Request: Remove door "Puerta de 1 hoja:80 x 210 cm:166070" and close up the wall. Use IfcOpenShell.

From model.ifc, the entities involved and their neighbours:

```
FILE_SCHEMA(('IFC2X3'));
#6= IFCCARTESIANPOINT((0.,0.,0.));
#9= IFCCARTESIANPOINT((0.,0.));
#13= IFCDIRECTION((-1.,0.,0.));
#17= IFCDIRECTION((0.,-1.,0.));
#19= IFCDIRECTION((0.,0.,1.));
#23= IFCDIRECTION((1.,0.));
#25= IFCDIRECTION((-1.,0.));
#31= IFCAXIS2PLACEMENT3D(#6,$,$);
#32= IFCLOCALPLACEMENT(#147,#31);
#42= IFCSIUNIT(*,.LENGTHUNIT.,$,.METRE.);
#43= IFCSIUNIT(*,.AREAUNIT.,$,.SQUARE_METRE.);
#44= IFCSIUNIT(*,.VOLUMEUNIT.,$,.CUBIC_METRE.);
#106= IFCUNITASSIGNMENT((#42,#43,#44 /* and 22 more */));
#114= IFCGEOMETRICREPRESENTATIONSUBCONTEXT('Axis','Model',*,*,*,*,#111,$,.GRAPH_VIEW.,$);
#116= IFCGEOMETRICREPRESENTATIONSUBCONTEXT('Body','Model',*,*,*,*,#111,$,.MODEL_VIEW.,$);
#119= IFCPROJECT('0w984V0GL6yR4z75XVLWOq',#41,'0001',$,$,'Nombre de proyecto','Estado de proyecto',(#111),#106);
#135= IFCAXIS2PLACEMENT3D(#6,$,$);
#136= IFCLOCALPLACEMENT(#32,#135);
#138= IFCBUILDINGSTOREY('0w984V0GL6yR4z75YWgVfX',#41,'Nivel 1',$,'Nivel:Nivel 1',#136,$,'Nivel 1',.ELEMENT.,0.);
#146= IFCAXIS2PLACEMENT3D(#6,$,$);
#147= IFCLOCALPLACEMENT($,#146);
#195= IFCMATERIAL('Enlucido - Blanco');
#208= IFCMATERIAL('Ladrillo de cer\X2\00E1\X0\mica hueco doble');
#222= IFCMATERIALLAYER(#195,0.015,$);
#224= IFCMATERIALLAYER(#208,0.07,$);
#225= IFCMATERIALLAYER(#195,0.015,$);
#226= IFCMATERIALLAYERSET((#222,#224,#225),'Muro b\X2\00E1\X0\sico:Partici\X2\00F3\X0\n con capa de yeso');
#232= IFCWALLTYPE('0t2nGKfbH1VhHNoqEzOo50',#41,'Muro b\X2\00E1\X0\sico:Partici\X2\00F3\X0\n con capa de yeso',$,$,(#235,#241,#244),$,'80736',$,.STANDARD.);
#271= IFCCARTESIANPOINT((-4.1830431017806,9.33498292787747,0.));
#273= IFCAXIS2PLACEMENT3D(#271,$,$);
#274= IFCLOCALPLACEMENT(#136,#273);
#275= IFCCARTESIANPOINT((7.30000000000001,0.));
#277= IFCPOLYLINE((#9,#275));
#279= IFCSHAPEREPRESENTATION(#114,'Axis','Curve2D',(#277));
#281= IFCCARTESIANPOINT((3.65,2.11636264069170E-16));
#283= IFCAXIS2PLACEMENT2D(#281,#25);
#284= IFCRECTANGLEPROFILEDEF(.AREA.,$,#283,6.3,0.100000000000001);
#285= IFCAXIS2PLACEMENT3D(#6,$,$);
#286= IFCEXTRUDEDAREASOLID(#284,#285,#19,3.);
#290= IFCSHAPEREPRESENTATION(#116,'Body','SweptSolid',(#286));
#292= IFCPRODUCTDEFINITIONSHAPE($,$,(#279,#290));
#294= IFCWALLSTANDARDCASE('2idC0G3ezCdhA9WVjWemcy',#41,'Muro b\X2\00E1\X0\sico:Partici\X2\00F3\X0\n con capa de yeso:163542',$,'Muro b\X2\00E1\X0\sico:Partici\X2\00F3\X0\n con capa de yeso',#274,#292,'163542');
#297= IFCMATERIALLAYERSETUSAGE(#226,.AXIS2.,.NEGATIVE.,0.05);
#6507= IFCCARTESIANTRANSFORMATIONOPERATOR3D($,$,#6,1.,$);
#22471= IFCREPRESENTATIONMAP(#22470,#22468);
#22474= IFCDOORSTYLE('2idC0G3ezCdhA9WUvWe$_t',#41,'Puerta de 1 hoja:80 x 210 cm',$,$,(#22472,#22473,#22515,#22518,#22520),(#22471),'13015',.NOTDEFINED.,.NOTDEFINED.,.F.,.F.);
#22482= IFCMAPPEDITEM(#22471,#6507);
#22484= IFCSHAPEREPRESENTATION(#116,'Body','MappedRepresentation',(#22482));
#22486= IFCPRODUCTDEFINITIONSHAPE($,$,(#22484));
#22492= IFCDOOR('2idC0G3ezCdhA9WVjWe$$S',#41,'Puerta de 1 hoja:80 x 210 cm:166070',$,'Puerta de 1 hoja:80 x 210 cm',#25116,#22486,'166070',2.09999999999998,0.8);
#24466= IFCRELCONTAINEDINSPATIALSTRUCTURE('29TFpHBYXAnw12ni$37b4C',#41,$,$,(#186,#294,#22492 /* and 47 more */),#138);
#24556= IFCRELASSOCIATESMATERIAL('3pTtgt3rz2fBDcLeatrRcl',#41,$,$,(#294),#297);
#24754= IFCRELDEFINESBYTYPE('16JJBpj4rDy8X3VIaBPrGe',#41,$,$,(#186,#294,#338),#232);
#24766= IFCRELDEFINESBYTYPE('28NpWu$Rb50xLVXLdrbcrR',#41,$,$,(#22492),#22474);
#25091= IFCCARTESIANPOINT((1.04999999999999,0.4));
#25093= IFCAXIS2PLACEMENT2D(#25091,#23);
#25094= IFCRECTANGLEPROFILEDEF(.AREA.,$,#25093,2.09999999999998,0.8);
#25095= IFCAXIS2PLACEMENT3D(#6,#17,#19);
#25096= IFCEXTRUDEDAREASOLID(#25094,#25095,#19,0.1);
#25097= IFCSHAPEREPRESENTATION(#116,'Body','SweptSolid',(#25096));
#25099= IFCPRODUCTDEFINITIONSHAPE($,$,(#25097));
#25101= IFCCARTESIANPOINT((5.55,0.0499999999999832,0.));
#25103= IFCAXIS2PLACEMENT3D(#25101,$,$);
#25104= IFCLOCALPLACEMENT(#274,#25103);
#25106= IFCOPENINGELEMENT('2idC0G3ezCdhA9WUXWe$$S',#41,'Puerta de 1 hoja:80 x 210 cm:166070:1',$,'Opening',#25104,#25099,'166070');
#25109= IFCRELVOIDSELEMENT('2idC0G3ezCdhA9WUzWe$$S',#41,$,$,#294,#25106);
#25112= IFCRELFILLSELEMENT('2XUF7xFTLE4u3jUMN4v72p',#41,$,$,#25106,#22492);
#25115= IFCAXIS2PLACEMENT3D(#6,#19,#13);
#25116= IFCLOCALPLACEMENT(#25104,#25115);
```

```python
import ifcopenshell
import ifcopenshell.api.feature
import ifcopenshell.api.root
import ifcopenshell.geom
import ifcopenshell.util.shape

model = ifcopenshell.open("model.ifc")
settings = ifcopenshell.geom.settings()


def volume(element):
    """Net volume in cubic metres, openings subtracted."""
    shape = ifcopenshell.geom.create_shape(settings, element)
    return ifcopenshell.util.shape.get_volume(shape.geometry)


door = model.by_id(22492)
opening = door.FillsVoids[0].RelatingOpeningElement
wall = opening.VoidsElements[0].RelatingBuildingElement
before = volume(wall)

ifcopenshell.api.root.remove_product(model, product=door)
ifcopenshell.api.feature.remove_feature(model, feature=opening)

after = volume(wall)

print(f"wall volume {before:.3f} -> {after:.3f} m3")

model.write("model_edited.ifc")
```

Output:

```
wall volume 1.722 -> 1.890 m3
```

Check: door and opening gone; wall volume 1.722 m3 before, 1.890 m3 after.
